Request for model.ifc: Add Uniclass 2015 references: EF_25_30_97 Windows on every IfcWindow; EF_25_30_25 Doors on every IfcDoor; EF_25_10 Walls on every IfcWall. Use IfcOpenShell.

First a look at what the model holds.

```python
import ifcopenshell

model = ifcopenshell.open("model.ifc")
print(model.schema)
print("classifications:", [c.Name for c in model.by_type("IfcClassification")])
for ifc_class in ("IfcDoor", "IfcRoof", "IfcStair", "IfcWall", "IfcWindow"):
    print(ifc_class, len(model.by_type(ifc_class)))
```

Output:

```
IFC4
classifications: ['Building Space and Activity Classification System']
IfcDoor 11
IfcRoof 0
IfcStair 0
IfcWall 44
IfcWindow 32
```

```python
import ifcopenshell
import ifcopenshell.api.classification

model = ifcopenshell.open("model.ifc")

system = ifcopenshell.api.classification.add_classification(model, classification="Uniclass 2015")

codes = {
    "IfcWindow": ("EF_25_30_97", "Windows"),
    "IfcDoor": ("EF_25_30_25", "Doors"),
    "IfcWall": ("EF_25_10", "Walls"),
}
for ifc_class, (code, name) in codes.items():
    products = model.by_type(ifc_class)
    ifcopenshell.api.classification.add_reference(
        model, products=products, classification=system, identification=code, name=name
    )
    print(code, len(products))

model.write("model_updated.ifc")
```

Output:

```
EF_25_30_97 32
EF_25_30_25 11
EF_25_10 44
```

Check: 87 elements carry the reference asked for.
